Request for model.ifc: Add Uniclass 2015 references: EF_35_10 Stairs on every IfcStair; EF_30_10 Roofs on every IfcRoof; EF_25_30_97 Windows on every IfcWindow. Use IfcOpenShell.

First a look at what the model holds.

```python
import ifcopenshell

model = ifcopenshell.open("model.ifc")
print(model.schema)
print("classifications:", [c.Name for c in model.by_type("IfcClassification")])
for ifc_class in ("IfcDoor", "IfcRoof", "IfcStair", "IfcWall", "IfcWindow"):
    print(ifc_class, len(model.by_type(ifc_class)))
```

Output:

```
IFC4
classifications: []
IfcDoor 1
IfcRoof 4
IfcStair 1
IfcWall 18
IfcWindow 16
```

```python
import ifcopenshell
import ifcopenshell.api.classification

model = ifcopenshell.open("model.ifc")

system = ifcopenshell.api.classification.add_classification(model, classification="Uniclass 2015")

codes = {
    "IfcStair": ("EF_35_10", "Stairs"),
    "IfcRoof": ("EF_30_10", "Roofs"),
    "IfcWindow": ("EF_25_30_97", "Windows"),
}
for ifc_class, (code, name) in codes.items():
    products = model.by_type(ifc_class)
    ifcopenshell.api.classification.add_reference(
        model, products=products, classification=system, identification=code, name=name
    )
    print(code, len(products))

model.write("model_v2.ifc")
```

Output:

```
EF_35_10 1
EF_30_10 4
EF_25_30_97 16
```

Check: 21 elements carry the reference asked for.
